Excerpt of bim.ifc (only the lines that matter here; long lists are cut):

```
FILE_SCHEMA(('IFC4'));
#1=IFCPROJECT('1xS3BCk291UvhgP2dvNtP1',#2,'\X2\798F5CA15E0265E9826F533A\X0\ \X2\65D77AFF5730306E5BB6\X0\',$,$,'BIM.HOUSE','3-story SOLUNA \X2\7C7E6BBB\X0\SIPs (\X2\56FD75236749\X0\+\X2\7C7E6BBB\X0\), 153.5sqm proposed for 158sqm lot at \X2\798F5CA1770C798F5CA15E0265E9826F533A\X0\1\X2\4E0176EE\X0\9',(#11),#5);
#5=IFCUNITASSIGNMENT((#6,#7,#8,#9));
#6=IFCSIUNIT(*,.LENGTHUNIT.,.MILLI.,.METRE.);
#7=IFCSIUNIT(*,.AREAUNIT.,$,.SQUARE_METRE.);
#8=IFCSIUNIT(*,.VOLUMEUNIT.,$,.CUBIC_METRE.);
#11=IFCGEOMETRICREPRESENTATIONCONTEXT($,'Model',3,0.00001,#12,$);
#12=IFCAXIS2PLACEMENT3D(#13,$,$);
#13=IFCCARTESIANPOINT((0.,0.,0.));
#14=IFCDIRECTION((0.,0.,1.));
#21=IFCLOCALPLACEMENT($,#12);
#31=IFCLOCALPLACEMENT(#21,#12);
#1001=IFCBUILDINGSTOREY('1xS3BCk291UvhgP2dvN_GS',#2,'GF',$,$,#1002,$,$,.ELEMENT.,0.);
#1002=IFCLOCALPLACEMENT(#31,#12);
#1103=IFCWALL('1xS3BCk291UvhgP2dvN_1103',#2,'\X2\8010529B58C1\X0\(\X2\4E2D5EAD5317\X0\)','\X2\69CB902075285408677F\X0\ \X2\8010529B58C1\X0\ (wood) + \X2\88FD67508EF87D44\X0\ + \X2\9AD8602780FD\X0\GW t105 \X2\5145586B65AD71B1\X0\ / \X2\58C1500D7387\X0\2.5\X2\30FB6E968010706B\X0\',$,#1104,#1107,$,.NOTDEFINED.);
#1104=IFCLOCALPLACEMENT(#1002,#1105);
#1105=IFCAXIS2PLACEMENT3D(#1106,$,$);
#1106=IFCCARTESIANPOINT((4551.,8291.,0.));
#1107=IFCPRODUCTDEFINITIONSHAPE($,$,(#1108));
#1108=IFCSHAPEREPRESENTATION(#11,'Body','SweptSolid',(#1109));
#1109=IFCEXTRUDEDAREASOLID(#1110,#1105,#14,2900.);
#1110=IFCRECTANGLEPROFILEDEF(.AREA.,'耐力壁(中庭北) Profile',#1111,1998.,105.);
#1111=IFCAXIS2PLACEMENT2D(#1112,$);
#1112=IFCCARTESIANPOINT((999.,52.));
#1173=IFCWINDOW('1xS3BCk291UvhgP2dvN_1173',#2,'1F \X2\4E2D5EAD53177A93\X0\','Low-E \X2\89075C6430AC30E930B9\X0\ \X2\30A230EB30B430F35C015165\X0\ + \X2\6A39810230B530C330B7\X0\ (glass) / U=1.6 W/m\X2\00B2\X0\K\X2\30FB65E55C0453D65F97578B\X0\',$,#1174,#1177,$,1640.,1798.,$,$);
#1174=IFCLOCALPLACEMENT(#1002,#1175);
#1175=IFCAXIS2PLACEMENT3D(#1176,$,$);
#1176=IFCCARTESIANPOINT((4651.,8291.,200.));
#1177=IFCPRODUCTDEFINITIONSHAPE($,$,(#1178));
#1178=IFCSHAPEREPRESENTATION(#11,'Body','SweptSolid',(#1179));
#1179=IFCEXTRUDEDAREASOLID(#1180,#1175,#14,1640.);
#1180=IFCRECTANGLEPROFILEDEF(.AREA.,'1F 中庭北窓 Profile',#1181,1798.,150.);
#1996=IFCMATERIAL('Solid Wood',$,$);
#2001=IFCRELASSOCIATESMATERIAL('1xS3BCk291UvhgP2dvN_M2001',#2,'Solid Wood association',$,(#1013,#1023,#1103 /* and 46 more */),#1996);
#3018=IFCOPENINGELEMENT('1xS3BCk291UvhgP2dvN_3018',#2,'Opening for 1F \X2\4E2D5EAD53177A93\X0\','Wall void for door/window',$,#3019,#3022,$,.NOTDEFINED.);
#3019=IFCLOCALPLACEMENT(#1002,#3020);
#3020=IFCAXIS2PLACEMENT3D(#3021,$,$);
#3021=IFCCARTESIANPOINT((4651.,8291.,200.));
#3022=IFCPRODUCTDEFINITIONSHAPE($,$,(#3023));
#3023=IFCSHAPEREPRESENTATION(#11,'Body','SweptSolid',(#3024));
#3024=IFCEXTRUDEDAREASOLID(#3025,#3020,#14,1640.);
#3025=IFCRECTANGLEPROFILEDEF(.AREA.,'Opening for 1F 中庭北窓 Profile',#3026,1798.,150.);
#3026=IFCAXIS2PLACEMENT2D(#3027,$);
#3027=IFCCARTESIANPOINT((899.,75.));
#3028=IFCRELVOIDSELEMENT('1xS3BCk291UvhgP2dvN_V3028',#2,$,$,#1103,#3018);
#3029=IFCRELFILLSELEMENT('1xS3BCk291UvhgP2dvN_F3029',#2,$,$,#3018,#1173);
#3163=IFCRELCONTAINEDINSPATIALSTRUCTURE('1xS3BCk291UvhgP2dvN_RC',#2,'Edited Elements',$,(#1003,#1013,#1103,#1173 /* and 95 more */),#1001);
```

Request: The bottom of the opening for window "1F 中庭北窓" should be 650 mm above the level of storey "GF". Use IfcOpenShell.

```python
import numpy as np
import ifcopenshell
import ifcopenshell.api.geometry
import ifcopenshell.geom
import ifcopenshell.util.element
import ifcopenshell.util.placement
import ifcopenshell.util.shape
import ifcopenshell.util.unit

model = ifcopenshell.open("bim.ifc")
unit_scale = ifcopenshell.util.unit.calculate_unit_scale(model)

window = model.by_guid("1xS3BCk291UvhgP2dvN_1173")
opening = window.FillsVoids[0].RelatingOpeningElement
storey = ifcopenshell.util.element.get_container(window, ifc_class="IfcBuildingStorey")
level = ifcopenshell.util.placement.get_local_placement(storey.ObjectPlacement)[2, 3]

# The opening's origin need not be at the sill, so measure its lowest point.
shape = ifcopenshell.geom.create_shape(ifcopenshell.geom.settings(), opening)
bottom = ifcopenshell.util.shape.get_shape_bottom_elevation(shape, shape.geometry) / unit_scale
dz = level + 650.0 - bottom

shift = np.array([0.0, 0.0, dz])
# The window is not placed relative to its opening, so move both.
for product in (opening, window):
    matrix = ifcopenshell.util.placement.get_local_placement(product.ObjectPlacement)
    matrix[:3, 3] += shift
    ifcopenshell.api.geometry.edit_object_placement(model, product=product, matrix=matrix, is_si=False)

print(f"moved by {dz * unit_scale:+.3f} m")

model.write("bim_v2.ifc")
```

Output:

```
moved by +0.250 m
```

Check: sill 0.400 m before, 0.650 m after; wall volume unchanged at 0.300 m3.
